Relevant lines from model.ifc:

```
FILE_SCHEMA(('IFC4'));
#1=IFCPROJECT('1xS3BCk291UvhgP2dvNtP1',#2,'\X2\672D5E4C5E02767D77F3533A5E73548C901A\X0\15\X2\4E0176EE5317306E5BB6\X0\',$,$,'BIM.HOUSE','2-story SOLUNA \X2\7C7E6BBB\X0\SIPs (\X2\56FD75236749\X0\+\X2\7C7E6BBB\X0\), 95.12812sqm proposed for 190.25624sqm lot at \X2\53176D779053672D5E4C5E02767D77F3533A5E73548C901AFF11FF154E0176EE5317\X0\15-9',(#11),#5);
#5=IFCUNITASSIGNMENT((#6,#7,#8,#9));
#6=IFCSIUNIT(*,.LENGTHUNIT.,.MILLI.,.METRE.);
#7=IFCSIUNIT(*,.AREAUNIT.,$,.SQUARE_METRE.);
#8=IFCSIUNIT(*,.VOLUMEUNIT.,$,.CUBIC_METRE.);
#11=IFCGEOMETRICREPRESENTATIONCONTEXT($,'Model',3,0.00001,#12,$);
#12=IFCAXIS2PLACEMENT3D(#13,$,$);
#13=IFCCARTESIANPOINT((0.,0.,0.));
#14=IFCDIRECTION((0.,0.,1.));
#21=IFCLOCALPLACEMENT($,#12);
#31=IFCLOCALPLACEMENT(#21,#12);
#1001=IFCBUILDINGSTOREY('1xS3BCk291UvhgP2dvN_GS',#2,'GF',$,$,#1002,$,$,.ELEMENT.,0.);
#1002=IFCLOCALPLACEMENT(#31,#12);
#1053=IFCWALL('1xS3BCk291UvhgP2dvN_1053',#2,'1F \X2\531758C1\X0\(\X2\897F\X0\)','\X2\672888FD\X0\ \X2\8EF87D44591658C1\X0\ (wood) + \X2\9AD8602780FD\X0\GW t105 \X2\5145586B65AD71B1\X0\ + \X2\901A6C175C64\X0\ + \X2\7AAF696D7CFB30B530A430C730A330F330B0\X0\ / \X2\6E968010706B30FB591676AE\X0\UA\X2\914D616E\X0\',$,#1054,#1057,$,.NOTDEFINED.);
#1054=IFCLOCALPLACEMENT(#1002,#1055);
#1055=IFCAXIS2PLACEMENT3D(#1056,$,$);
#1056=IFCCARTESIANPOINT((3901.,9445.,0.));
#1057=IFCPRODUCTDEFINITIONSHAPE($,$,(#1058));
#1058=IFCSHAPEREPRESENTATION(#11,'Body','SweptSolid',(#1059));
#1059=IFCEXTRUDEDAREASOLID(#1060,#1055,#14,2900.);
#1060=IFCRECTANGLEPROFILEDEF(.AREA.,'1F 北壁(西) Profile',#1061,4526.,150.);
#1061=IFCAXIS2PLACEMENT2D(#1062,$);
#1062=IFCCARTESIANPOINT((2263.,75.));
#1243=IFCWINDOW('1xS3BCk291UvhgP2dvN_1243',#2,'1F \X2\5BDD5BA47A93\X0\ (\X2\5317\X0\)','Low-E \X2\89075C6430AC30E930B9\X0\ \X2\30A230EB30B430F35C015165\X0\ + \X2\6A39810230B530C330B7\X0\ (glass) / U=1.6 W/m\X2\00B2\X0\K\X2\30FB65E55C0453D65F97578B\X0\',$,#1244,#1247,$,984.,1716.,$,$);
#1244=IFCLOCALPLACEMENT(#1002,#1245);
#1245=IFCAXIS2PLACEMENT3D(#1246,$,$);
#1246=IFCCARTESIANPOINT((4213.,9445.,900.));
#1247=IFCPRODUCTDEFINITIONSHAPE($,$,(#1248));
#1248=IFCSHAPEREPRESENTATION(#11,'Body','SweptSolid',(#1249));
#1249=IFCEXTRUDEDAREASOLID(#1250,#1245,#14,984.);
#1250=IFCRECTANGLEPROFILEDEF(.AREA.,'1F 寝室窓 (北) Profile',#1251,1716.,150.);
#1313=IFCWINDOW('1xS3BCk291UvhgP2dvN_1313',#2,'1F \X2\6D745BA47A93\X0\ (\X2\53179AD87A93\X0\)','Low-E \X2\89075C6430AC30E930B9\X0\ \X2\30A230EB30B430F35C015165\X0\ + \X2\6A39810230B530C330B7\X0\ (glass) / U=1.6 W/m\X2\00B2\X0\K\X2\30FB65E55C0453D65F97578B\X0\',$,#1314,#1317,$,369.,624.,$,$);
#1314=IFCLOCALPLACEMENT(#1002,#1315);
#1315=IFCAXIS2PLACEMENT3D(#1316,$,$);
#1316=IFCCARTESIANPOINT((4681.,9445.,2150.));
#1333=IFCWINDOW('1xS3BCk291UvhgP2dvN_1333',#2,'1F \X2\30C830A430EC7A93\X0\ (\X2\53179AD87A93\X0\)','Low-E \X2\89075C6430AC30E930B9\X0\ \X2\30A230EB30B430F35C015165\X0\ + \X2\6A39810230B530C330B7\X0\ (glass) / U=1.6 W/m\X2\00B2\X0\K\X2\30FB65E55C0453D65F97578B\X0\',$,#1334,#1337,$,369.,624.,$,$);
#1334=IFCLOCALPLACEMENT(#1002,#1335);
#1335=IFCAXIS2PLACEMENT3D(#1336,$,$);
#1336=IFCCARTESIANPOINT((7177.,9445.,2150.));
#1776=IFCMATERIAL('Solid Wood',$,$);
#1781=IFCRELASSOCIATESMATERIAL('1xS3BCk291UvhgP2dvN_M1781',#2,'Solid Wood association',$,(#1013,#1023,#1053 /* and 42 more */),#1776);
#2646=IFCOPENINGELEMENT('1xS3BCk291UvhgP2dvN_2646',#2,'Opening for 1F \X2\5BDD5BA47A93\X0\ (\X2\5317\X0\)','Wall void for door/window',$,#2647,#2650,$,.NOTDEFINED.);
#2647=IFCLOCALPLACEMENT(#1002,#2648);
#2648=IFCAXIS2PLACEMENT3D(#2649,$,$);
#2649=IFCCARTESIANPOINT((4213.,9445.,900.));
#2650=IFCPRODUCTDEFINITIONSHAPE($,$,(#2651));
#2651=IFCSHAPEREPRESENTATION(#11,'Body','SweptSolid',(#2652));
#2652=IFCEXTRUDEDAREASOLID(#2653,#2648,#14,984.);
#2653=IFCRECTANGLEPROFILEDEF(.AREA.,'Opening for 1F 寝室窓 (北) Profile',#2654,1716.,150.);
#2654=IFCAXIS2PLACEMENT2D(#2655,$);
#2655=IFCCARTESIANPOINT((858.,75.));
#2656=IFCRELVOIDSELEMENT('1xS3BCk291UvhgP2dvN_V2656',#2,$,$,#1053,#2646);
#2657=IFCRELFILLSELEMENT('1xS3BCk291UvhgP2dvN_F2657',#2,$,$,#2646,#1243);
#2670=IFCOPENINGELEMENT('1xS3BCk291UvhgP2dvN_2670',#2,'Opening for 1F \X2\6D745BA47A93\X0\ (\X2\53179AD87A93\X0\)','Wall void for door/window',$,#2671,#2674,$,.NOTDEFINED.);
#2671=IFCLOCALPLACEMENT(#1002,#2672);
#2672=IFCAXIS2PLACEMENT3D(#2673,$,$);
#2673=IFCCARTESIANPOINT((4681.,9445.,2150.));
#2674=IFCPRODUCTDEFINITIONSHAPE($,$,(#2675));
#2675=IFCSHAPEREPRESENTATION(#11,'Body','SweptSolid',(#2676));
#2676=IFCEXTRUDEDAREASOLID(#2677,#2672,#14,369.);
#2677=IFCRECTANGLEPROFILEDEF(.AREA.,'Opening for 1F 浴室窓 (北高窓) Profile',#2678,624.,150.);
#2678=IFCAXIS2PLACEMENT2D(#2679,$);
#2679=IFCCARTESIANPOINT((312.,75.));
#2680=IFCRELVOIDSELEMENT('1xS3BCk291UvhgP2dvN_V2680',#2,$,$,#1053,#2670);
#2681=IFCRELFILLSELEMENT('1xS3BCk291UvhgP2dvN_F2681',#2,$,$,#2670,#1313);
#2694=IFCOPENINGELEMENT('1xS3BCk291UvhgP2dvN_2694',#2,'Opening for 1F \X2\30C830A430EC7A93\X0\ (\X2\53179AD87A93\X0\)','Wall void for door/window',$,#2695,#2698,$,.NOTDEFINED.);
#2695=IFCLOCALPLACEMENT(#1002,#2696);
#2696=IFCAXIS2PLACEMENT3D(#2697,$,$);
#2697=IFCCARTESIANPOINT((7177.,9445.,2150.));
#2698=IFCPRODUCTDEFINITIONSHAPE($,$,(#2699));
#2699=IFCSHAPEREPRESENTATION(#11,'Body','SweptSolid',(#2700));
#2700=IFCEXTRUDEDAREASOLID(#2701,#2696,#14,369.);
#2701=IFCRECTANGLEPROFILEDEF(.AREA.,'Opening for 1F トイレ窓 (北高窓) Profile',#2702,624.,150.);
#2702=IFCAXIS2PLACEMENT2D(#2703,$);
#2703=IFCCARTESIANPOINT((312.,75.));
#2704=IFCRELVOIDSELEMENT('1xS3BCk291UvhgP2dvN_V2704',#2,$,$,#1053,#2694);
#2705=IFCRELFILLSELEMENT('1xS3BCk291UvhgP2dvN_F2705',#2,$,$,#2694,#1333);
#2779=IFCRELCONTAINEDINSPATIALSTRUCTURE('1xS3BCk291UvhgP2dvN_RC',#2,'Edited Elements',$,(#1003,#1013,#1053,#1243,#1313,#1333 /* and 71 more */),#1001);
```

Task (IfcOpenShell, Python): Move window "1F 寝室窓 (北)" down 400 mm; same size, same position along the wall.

```python
import numpy as np
import ifcopenshell
import ifcopenshell.api.geometry
import ifcopenshell.util.placement
import ifcopenshell.util.unit

model = ifcopenshell.open("model.ifc")
unit_scale = ifcopenshell.util.unit.calculate_unit_scale(model)

window = model.by_guid("1xS3BCk291UvhgP2dvN_1243")
opening = window.FillsVoids[0].RelatingOpeningElement
dz = -400.0

shift = np.array([0.0, 0.0, dz])
# The window is not placed relative to its opening, so move both.
for product in (opening, window):
    matrix = ifcopenshell.util.placement.get_local_placement(product.ObjectPlacement)
    matrix[:3, 3] += shift
    ifcopenshell.api.geometry.edit_object_placement(model, product=product, matrix=matrix, is_si=False)

print(f"moved by {dz * unit_scale:+.3f} m")

model.write("model-out.ifc")
```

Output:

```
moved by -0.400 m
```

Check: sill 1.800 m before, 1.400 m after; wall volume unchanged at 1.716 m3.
